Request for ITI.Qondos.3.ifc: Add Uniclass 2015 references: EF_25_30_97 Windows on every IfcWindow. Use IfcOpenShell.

First a look at what the model holds.

```python
import ifcopenshell

model = ifcopenshell.open("ITI.Qondos.3.ifc")
print(model.schema)
print("classifications:", [c.Name for c in model.by_type("IfcClassification")])
for ifc_class in ("IfcDoor", "IfcRoof", "IfcStair", "IfcWall", "IfcWindow"):
    print(ifc_class, len(model.by_type(ifc_class)))
```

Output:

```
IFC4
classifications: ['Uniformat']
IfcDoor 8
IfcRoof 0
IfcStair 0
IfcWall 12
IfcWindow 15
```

```python
import ifcopenshell
import ifcopenshell.api.classification

model = ifcopenshell.open("ITI.Qondos.3.ifc")

system = ifcopenshell.api.classification.add_classification(model, classification="Uniclass 2015")

codes = {
    "IfcWindow": ("EF_25_30_97", "Windows"),
}
for ifc_class, (code, name) in codes.items():
    products = model.by_type(ifc_class)
    ifcopenshell.api.classification.add_reference(
        model, products=products, classification=system, identification=code, name=name
    )
    print(code, len(products))

model.write("ITI.Qondos.3_edited.ifc")
```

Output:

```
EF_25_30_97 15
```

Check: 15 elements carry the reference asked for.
